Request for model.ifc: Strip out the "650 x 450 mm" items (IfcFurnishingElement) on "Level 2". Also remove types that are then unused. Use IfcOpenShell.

First a look at what the model holds.

```python
import ifcopenshell
import ifcopenshell.util.element

model = ifcopenshell.open("model.ifc")
print(model.schema)
storey = next(s for s in model.by_type("IfcBuildingStorey") if s.Name == "Level 2")
furniture = [e for e in ifcopenshell.util.element.get_decomposition(storey) if e.is_a("IfcFurnishingElement")]
seen = {}
for e in furniture:
    element_type = ifcopenshell.util.element.get_type(e)
    name = element_type.Name if element_type not in (None, e) else None
    seen[name] = seen.get(name, 0) + 1
for name, count in sorted(seen.items(), key=str):
    print(count, "x", name)
```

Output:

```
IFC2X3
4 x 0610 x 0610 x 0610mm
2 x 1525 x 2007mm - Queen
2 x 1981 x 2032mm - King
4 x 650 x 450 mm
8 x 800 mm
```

```python
import ifcopenshell
import ifcopenshell.api.root
import ifcopenshell.util.element

model = ifcopenshell.open("model.ifc")

storey = next(s for s in model.by_type("IfcBuildingStorey") if s.Name == "Level 2")
furniture = [e for e in ifcopenshell.util.element.get_decomposition(storey) if e.is_a("IfcFurnishingElement")]
targets = [e for e in furniture if (t := ifcopenshell.util.element.get_type(e)) not in (None, e) and t.Name == "650 x 450 mm"]
types = {ifcopenshell.util.element.get_type(e) for e in targets} - {None, *targets}

for e in targets:
    ifcopenshell.api.root.remove_product(model, product=e)
print(len(targets), "removed")

unused = [t for t in types if not ifcopenshell.util.element.get_types(t)]
for t in unused:
    ifcopenshell.api.root.remove_product(model, product=t)
print(len(unused), "unused types removed")

model.write("model_edited.ifc")
```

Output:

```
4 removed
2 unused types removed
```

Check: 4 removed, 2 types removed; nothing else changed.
